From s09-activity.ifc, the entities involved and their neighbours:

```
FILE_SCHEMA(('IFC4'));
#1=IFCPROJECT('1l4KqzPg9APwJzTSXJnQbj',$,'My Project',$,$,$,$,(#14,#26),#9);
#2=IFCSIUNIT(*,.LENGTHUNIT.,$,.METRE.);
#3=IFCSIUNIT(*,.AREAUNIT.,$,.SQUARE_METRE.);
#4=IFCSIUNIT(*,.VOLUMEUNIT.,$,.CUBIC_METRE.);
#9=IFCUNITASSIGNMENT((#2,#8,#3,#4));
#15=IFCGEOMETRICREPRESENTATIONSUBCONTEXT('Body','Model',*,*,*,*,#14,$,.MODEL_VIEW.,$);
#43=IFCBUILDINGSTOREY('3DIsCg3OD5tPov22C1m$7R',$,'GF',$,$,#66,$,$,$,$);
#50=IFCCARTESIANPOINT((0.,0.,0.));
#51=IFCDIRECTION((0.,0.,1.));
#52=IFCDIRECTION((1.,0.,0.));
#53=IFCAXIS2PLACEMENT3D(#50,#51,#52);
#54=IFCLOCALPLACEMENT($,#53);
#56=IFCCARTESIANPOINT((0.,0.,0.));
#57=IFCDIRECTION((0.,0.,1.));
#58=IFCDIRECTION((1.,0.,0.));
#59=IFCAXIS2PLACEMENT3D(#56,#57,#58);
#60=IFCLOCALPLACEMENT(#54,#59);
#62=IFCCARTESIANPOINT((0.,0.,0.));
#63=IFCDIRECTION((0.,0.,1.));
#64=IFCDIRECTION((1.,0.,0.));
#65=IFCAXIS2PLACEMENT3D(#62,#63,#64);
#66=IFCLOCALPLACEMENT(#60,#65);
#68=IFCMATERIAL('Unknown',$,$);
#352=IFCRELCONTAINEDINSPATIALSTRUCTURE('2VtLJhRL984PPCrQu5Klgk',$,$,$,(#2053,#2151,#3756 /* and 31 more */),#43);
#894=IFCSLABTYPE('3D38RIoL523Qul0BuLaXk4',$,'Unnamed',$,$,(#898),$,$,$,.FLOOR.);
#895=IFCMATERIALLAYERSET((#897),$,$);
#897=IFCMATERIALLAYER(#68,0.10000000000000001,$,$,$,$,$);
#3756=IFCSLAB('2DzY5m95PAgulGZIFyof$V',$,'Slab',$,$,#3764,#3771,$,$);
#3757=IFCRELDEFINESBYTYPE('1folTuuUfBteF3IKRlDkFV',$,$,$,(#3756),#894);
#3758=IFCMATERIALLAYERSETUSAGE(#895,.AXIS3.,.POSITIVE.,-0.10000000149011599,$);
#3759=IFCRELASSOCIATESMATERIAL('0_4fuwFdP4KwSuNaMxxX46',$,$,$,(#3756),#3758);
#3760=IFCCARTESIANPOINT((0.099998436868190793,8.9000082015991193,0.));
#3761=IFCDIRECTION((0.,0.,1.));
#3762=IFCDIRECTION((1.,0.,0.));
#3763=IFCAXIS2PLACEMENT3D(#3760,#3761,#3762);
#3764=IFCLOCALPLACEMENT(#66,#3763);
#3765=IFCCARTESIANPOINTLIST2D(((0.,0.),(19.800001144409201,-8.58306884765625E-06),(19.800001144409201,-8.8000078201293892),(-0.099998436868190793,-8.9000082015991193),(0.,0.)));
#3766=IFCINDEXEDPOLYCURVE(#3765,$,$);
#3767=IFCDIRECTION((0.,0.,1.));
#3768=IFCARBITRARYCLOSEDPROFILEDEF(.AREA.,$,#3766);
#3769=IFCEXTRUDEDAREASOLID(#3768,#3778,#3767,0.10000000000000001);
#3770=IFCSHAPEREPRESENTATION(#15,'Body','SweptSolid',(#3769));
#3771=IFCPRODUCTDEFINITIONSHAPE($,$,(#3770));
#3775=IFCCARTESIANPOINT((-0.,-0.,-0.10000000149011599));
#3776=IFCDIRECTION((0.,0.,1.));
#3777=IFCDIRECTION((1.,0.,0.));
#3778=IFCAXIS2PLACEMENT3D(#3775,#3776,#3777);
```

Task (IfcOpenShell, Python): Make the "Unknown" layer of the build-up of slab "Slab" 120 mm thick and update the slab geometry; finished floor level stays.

```python
import ifcopenshell
import ifcopenshell.util.element
import ifcopenshell.util.representation

model = ifcopenshell.open("s09-activity.ifc")

layer_set = model.by_id(895)
layer = next(l for l in layer_set.MaterialLayers if l.Material and l.Material.Name == "Unknown")
change = 0.12 - layer.LayerThickness
layer.LayerThickness += change

# Geometry does not follow the layer set by itself.
slabs = [e for e in ifcopenshell.util.element.get_elements_by_material(model, layer_set) if e.is_a("IfcSlab")]
for slab in sorted(slabs, key=lambda e: e.id()):
    body = ifcopenshell.util.representation.get_representation(slab, "Model", "Body")
    solid = body.Items[0]
    old_depth = solid.Depth
    solid.Depth += change
    # Extruded upwards: lower the start of the extrusion so the top stays.
    x, y, z = solid.Position.Location.Coordinates
    solid.Position.Location = model.createIfcCartesianPoint((x, y, z - change))
    print(slab.id(), f"{old_depth:g} -> {solid.Depth:g}")

# The layers are counted up from the underside, which has moved.
for usage in {ifcopenshell.util.element.get_material(slab) for slab in slabs}:
    usage.OffsetFromReferenceLine -= change

model.write("s09-activity-out.ifc")
```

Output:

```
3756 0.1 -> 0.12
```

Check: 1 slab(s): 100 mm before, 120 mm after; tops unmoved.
